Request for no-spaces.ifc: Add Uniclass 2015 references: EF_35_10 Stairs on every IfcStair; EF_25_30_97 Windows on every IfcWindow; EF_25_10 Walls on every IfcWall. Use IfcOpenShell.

First a look at what the model holds.

```python
import ifcopenshell

model = ifcopenshell.open("no-spaces.ifc")
print(model.schema)
print("classifications:", [c.Name for c in model.by_type("IfcClassification")])
for ifc_class in ("IfcDoor", "IfcRoof", "IfcStair", "IfcWall", "IfcWindow"):
    print(ifc_class, len(model.by_type(ifc_class)))
```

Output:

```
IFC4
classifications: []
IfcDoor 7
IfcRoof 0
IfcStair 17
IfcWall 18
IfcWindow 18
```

```python
import ifcopenshell
import ifcopenshell.api.classification

model = ifcopenshell.open("no-spaces.ifc")

system = ifcopenshell.api.classification.add_classification(model, classification="Uniclass 2015")

codes = {
    "IfcStair": ("EF_35_10", "Stairs"),
    "IfcWindow": ("EF_25_30_97", "Windows"),
    "IfcWall": ("EF_25_10", "Walls"),
}
for ifc_class, (code, name) in codes.items():
    products = model.by_type(ifc_class)
    ifcopenshell.api.classification.add_reference(
        model, products=products, classification=system, identification=code, name=name
    )
    print(code, len(products))

model.write("no-spaces_updated.ifc")
```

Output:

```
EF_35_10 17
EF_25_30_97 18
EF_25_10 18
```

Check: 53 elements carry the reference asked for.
